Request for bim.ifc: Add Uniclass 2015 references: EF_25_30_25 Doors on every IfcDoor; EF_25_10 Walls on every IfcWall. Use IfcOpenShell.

First a look at what the model holds.

```python
import ifcopenshell

model = ifcopenshell.open("bim.ifc")
print(model.schema)
print("classifications:", [c.Name for c in model.by_type("IfcClassification")])
for ifc_class in ("IfcDoor", "IfcRoof", "IfcStair", "IfcWall", "IfcWindow"):
    print(ifc_class, len(model.by_type(ifc_class)))
```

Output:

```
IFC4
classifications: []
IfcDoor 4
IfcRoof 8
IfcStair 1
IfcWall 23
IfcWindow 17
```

```python
import ifcopenshell
import ifcopenshell.api.classification

model = ifcopenshell.open("bim.ifc")

system = ifcopenshell.api.classification.add_classification(model, classification="Uniclass 2015")

codes = {
    "IfcDoor": ("EF_25_30_25", "Doors"),
    "IfcWall": ("EF_25_10", "Walls"),
}
for ifc_class, (code, name) in codes.items():
    products = model.by_type(ifc_class)
    ifcopenshell.api.classification.add_reference(
        model, products=products, classification=system, identification=code, name=name
    )
    print(code, len(products))

model.write("bim_rev.ifc")
```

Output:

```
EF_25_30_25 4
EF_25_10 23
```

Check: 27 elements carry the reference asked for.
